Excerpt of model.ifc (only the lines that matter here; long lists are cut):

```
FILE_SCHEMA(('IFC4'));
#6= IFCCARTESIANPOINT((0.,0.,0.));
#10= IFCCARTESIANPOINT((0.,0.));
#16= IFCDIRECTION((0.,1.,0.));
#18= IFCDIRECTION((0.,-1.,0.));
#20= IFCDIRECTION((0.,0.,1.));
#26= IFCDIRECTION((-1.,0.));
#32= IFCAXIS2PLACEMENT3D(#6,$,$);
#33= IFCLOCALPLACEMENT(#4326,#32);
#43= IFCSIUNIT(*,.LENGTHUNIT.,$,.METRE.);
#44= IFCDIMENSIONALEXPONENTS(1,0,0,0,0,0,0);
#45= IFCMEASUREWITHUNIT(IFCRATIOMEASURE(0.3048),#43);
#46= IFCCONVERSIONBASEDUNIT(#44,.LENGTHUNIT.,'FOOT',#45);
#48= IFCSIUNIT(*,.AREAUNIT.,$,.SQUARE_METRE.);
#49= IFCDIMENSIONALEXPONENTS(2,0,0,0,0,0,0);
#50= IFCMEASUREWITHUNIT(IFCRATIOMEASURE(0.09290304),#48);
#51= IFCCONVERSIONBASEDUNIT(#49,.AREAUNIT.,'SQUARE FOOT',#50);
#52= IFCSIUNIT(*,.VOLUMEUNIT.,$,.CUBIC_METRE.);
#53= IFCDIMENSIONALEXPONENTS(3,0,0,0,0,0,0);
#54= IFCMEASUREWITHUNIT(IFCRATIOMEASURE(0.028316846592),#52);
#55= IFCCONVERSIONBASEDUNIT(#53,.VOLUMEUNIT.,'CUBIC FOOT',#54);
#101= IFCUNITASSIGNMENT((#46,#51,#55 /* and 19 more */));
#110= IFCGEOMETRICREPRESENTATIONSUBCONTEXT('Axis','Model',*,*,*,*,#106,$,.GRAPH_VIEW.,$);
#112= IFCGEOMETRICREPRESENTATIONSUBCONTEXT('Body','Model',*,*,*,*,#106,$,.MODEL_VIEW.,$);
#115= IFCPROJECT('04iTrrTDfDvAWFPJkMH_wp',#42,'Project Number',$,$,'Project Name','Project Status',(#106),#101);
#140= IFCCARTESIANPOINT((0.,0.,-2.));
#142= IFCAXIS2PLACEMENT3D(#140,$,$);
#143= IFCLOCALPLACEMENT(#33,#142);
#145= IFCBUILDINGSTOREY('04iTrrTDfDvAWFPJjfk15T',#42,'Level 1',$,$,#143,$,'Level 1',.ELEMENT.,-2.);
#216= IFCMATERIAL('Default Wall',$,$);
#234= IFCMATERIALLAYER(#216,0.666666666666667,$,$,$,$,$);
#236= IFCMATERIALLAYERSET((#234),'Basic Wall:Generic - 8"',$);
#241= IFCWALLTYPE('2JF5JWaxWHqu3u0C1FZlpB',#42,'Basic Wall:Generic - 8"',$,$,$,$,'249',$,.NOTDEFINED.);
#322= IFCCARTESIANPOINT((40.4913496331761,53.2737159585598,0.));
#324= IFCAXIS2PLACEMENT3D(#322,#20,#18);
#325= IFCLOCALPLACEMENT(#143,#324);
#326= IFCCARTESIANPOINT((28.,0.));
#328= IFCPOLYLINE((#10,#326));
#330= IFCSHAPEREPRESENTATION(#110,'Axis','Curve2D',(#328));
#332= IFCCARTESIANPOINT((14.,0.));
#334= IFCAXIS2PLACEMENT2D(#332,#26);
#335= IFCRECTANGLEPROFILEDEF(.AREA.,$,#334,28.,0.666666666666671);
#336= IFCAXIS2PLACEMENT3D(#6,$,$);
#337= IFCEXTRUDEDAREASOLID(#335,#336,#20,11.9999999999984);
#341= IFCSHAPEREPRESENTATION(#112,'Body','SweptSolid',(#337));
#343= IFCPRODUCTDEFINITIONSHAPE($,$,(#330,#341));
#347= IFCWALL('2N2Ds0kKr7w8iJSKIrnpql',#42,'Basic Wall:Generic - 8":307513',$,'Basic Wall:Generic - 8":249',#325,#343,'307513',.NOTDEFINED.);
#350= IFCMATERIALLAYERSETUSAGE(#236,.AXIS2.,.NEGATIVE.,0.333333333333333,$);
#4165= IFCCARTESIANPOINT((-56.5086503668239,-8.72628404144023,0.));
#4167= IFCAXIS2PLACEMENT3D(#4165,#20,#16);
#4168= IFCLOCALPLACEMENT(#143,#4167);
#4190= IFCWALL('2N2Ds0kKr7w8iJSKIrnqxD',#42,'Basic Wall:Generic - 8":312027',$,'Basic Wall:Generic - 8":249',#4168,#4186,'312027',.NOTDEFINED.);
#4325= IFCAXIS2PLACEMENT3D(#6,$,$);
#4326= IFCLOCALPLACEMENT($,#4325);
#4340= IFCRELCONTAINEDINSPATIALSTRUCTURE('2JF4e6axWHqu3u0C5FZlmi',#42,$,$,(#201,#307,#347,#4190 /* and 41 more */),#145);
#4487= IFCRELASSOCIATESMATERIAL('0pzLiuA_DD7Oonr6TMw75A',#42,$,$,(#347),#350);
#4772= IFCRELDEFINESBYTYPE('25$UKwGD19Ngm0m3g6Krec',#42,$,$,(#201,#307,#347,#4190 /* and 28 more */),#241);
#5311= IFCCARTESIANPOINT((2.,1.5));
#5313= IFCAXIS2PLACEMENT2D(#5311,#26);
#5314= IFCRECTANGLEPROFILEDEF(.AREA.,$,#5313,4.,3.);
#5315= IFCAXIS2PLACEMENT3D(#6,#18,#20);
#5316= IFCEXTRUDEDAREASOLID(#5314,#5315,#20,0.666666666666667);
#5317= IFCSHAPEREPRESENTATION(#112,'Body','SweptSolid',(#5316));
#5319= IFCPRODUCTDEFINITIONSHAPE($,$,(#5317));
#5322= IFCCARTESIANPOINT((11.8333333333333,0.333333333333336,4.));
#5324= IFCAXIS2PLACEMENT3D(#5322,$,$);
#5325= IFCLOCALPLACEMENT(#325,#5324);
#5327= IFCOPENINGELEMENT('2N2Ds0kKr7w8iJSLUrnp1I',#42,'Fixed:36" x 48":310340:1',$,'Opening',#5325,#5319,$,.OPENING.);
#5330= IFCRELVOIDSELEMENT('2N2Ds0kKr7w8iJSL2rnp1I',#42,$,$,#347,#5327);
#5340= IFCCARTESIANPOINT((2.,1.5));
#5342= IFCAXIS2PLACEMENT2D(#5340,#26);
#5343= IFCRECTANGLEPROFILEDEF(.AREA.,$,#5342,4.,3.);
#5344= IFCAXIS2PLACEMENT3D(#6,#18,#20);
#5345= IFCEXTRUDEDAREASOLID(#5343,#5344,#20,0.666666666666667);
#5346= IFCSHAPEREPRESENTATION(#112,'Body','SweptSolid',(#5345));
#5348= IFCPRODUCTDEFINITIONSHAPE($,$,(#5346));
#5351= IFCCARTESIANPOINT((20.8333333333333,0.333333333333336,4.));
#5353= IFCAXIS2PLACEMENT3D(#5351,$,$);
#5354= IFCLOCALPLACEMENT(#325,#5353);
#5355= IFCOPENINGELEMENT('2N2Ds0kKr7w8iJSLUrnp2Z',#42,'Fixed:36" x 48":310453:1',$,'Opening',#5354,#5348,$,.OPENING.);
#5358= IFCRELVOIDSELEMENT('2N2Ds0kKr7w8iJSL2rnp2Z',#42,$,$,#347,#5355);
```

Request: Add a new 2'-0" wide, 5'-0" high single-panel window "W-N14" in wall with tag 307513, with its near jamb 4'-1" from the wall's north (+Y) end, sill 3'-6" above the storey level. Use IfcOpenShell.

```python
import numpy as np
import ifcopenshell
import ifcopenshell.api.feature
import ifcopenshell.api.geometry
import ifcopenshell.api.root
import ifcopenshell.api.spatial
import ifcopenshell.geom
import ifcopenshell.util.element
import ifcopenshell.util.placement
import ifcopenshell.util.representation
import ifcopenshell.util.shape
import ifcopenshell.util.unit

model = ifcopenshell.open("model.ifc")
unit_scale = ifcopenshell.util.unit.calculate_unit_scale(model)
settings = ifcopenshell.geom.settings()


def volume(element):
    """Net volume in cubic metres, openings subtracted."""
    shape = ifcopenshell.geom.create_shape(settings, element)
    return ifcopenshell.util.shape.get_volume(shape.geometry)


wall = model.by_guid("2N2Ds0kKr7w8iJSKIrnpql")
storey = ifcopenshell.util.element.get_container(wall, ifc_class="IfcBuildingStorey")
context = ifcopenshell.util.representation.get_context(model, "Model", "Body", "MODEL_VIEW")
before = volume(wall)

width, height, from_end, sill = 0.6096, 1.524, 1.2446, 1.0668  # metres

# The wall runs along its own X axis, and the end named is its -X end.
wall_shape = ifcopenshell.geom.create_shape(settings, wall)
x, y, z = ifcopenshell.util.shape.get_vertices(wall_shape.geometry).T
start = x.min() + from_end
face, thickness = float(y.min()), float(y.max() - y.min())
wall_matrix = ifcopenshell.util.placement.get_local_placement(wall.ObjectPlacement)
level = ifcopenshell.util.placement.get_local_placement(storey.ObjectPlacement)[2, 3]


def in_wall(x, y):
    """Placement at x, y metres in the wall's axes, at sill height."""
    matrix = wall_matrix.copy()
    matrix[:, 3] = wall_matrix @ np.array([x / unit_scale, y / unit_scale, 0.0, 1.0])
    matrix[2, 3] = level + sill / unit_scale
    return matrix


# Opening: a box that overshoots both wall faces by 50 mm.
opening = ifcopenshell.api.root.create_entity(model, ifc_class="IfcOpeningElement", predefined_type="OPENING")
box = ifcopenshell.api.geometry.add_wall_representation(
    model, context=context, length=width, height=height, thickness=thickness + 0.1
)
ifcopenshell.api.geometry.assign_representation(model, product=opening, representation=box)
ifcopenshell.api.geometry.edit_object_placement(model, product=opening, matrix=in_wall(start, face - 0.05), is_si=False)
ifcopenshell.api.feature.add_feature(model, feature=opening, element=wall)

window = ifcopenshell.api.root.create_entity(model, ifc_class="IfcWindow", name="W-N14", predefined_type="WINDOW")
window.OverallWidth, window.OverallHeight = width / unit_scale, height / unit_scale
window.PartitioningType = "SINGLE_PANEL"
body = ifcopenshell.api.geometry.add_window_representation(
    model,
    context=context,
    overall_width=window.OverallWidth,
    overall_height=window.OverallHeight,
    partition_type="SINGLE_PANEL",
)
ifcopenshell.api.geometry.assign_representation(model, product=window, representation=body)
ifcopenshell.api.spatial.assign_container(model, products=[window], relating_structure=storey)
ifcopenshell.api.feature.add_filling(model, opening=opening, element=window)

# Centre the window in the wall's thickness.
ifcopenshell.api.geometry.edit_object_placement(model, product=window, matrix=in_wall(start, face), is_si=False)
window_shape = ifcopenshell.geom.create_shape(settings, window)
depth = ifcopenshell.util.shape.get_vertices(window_shape.geometry)[:, 1]
offset = face + thickness / 2 - (depth.min() + depth.max()) / 2
ifcopenshell.api.geometry.edit_object_placement(model, product=window, matrix=in_wall(start, offset), is_si=False)

after = volume(wall)

print(f"wall volume {before:.3f} -> {after:.3f} m3")

model.write("model_v2.ifc")
```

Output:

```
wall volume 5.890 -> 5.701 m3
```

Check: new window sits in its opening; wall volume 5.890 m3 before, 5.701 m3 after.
